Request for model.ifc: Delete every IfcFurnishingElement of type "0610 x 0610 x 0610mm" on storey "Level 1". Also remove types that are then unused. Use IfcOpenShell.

First a look at what the model holds.

```python
import ifcopenshell
import ifcopenshell.util.element

model = ifcopenshell.open("model.ifc")
print(model.schema)
storey = next(s for s in model.by_type("IfcBuildingStorey") if s.Name == "Level 1")
furniture = [e for e in ifcopenshell.util.element.get_decomposition(storey) if e.is_a("IfcFurnishingElement")]
seen = {}
for e in furniture:
    element_type = ifcopenshell.util.element.get_type(e)
    name = element_type.Name if element_type not in (None, e) else None
    seen[name] = seen.get(name, 0) + 1
for name, count in sorted(seen.items(), key=str):
    print(count, "x", name)
```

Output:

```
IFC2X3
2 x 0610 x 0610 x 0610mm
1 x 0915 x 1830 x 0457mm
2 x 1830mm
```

```python
import ifcopenshell
import ifcopenshell.api.root
import ifcopenshell.util.element

model = ifcopenshell.open("model.ifc")

storey = next(s for s in model.by_type("IfcBuildingStorey") if s.Name == "Level 1")
furniture = [e for e in ifcopenshell.util.element.get_decomposition(storey) if e.is_a("IfcFurnishingElement")]
targets = [e for e in furniture if (t := ifcopenshell.util.element.get_type(e)) not in (None, e) and t.Name == "0610 x 0610 x 0610mm"]
types = {ifcopenshell.util.element.get_type(e) for e in targets} - {None, *targets}

for e in targets:
    ifcopenshell.api.root.remove_product(model, product=e)
print(len(targets), "removed")

unused = [t for t in types if not ifcopenshell.util.element.get_types(t)]
for t in unused:
    ifcopenshell.api.root.remove_product(model, product=t)
print(len(unused), "unused types removed")

model.write("model_updated.ifc")
```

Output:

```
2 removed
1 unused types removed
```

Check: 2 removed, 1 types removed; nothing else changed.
